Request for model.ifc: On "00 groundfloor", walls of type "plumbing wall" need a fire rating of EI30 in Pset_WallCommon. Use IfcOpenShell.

First a look at what the model holds.

```python
import ifcopenshell
import ifcopenshell.util.element

model = ifcopenshell.open("model.ifc")
print(model.schema)
storey = next(s for s in model.by_type("IfcBuildingStorey") if s.Name == "00 groundfloor")
walls = [e for e in ifcopenshell.util.element.get_decomposition(storey) if e.is_a("IfcWall")]
seen = {}
for e in walls:
    element_type = ifcopenshell.util.element.get_type(e)
    key = (element_type.Name if element_type != e and element_type else None, ifcopenshell.util.element.get_pset(e, "Pset_WallCommon", "FireRating"))
    seen[key] = seen.get(key, 0) + 1
for (name, value), count in sorted(seen.items(), key=str):
    print(count, "x", name, "|", value)
```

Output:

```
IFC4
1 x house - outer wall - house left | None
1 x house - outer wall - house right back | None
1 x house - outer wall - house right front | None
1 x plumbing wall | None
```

```python
import ifcopenshell
import ifcopenshell.api.pset
import ifcopenshell.util.element

model = ifcopenshell.open("model.ifc")

storey = next(s for s in model.by_type("IfcBuildingStorey") if s.Name == "00 groundfloor")
walls = [e for e in ifcopenshell.util.element.get_decomposition(storey) if e.is_a("IfcWall")]

count = 0
for e in walls:
    element_type = ifcopenshell.util.element.get_type(e)
    if element_type in (None, e) or element_type.Name != "plumbing wall":
        continue
    # add_pset returns the element's existing set when there is one.
    pset = ifcopenshell.api.pset.add_pset(model, product=e, name="Pset_WallCommon")
    ifcopenshell.api.pset.edit_pset(model, pset=pset, properties={"FireRating": "EI30"})
    count += 1

print(count, "walls updated")

model.write("model_edited.ifc")
```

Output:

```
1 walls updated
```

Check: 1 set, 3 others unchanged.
